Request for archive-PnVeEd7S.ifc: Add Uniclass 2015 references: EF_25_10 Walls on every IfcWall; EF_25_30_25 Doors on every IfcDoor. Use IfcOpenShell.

First a look at what the model holds.

```python
import ifcopenshell

model = ifcopenshell.open("archive-PnVeEd7S.ifc")
print(model.schema)
print("classifications:", [c.Name for c in model.by_type("IfcClassification")])
for ifc_class in ("IfcDoor", "IfcRoof", "IfcStair", "IfcWall", "IfcWindow"):
    print(ifc_class, len(model.by_type(ifc_class)))
```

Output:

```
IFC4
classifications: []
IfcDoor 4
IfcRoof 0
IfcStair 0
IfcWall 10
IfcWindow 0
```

```python
import ifcopenshell
import ifcopenshell.api.classification

model = ifcopenshell.open("archive-PnVeEd7S.ifc")

system = ifcopenshell.api.classification.add_classification(model, classification="Uniclass 2015")

codes = {
    "IfcWall": ("EF_25_10", "Walls"),
    "IfcDoor": ("EF_25_30_25", "Doors"),
}
for ifc_class, (code, name) in codes.items():
    products = model.by_type(ifc_class)
    ifcopenshell.api.classification.add_reference(
        model, products=products, classification=system, identification=code, name=name
    )
    print(code, len(products))

model.write("archive-PnVeEd7S_updated.ifc")
```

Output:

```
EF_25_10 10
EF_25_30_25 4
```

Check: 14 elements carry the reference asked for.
